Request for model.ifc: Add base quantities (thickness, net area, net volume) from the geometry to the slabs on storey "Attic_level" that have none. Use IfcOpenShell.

First a look at what the model holds.

```python
import ifcopenshell
import ifcopenshell.util.element
import ifcopenshell.util.unit

model = ifcopenshell.open("model.ifc")
print(model.schema)
for unit_type in ("LENGTHUNIT", "AREAUNIT", "VOLUMEUNIT"):
    print(unit_type, ifcopenshell.util.unit.calculate_unit_scale(model, unit_type))
storey = next(s for s in model.by_type("IfcBuildingStorey") if s.Name == "Attic_level")
slabs = [e for e in ifcopenshell.util.element.get_decomposition(storey) if e.is_a("IfcSlab")]
for e in sorted(slabs, key=lambda e: e.id()):
    print(e.id(), e.is_a(), e.Name, list(ifcopenshell.util.element.get_psets(e, qtos_only=True)), sep=" | ")
```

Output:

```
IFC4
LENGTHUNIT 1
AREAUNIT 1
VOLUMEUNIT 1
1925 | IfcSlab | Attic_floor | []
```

```python
import ifcopenshell
import ifcopenshell.api.pset
import ifcopenshell.geom
import ifcopenshell.util.element
import ifcopenshell.util.shape
import ifcopenshell.util.unit

model = ifcopenshell.open("model.ifc")
unit_scale = ifcopenshell.util.unit.calculate_unit_scale(model)
area_scale = ifcopenshell.util.unit.calculate_unit_scale(model, "AREAUNIT")
volume_scale = ifcopenshell.util.unit.calculate_unit_scale(model, "VOLUMEUNIT")
settings = ifcopenshell.geom.settings()

storey = next(s for s in model.by_type("IfcBuildingStorey") if s.Name == "Attic_level")
slabs = [e for e in ifcopenshell.util.element.get_decomposition(storey) if e.is_a("IfcSlab")]

for e in sorted(slabs, key=lambda e: e.id()):
    if ifcopenshell.util.element.get_psets(e, qtos_only=True, should_inherit=False):
        continue
    # Geometry comes back in metres, in the element's own axes.
    shape = ifcopenshell.geom.create_shape(settings, e)
    values = {
        "Width": ifcopenshell.util.shape.get_z(shape.geometry) / unit_scale,
        "NetArea": ifcopenshell.util.shape.get_footprint_area(shape.geometry) / area_scale,
        "NetVolume": ifcopenshell.util.shape.get_volume(shape.geometry) / volume_scale,
    }
    qto = ifcopenshell.api.pset.add_qto(model, product=e, name="Qto_SlabBaseQuantities")
    ifcopenshell.api.pset.edit_qto(model, qto=qto, properties=values)
    print(e.id(), {k: round(v, 3) for k, v in values.items()})

model.write("model_updated.ifc")
```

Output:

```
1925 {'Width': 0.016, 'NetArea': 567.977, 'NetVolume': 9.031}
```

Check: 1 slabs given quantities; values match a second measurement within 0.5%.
